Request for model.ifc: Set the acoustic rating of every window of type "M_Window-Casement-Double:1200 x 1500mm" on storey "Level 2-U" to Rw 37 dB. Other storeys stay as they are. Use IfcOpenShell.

First a look at what the model holds.

```python
import ifcopenshell
import ifcopenshell.util.element

model = ifcopenshell.open("model.ifc")
print(model.schema)
storey = next(s for s in model.by_type("IfcBuildingStorey") if s.Name == "Level 2-U")
windows = [e for e in ifcopenshell.util.element.get_decomposition(storey) if e.is_a("IfcWindow")]
seen = {}
for e in windows:
    element_type = ifcopenshell.util.element.get_type(e)
    key = (element_type.Name if element_type != e and element_type else None, ifcopenshell.util.element.get_pset(e, "Pset_WindowCommon", "AcousticRating"))
    seen[key] = seen.get(key, 0) + 1
for (name, value), count in sorted(seen.items(), key=str):
    print(count, "x", name, "|", value)
```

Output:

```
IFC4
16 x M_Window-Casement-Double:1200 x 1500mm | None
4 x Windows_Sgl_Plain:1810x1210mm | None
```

```python
import ifcopenshell
import ifcopenshell.api.pset
import ifcopenshell.util.element

model = ifcopenshell.open("model.ifc")

storey = next(s for s in model.by_type("IfcBuildingStorey") if s.Name == "Level 2-U")
windows = [e for e in ifcopenshell.util.element.get_decomposition(storey) if e.is_a("IfcWindow")]

count = 0
for e in windows:
    element_type = ifcopenshell.util.element.get_type(e)
    if element_type in (None, e) or element_type.Name != "M_Window-Casement-Double:1200 x 1500mm":
        continue
    # add_pset returns the element's existing set when there is one.
    pset = ifcopenshell.api.pset.add_pset(model, product=e, name="Pset_WindowCommon")
    ifcopenshell.api.pset.edit_pset(model, pset=pset, properties={"AcousticRating": "Rw 37 dB"})
    count += 1

print(count, "windows updated")

model.write("model_v2.ifc")
```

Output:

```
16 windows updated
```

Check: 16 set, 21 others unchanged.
